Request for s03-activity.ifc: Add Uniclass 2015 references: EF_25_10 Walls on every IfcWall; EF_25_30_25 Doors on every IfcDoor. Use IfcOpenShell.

First a look at what the model holds.

```python
import ifcopenshell

model = ifcopenshell.open("s03-activity.ifc")
print(model.schema)
print("classifications:", [c.Name for c in model.by_type("IfcClassification")])
for ifc_class in ("IfcDoor", "IfcRoof", "IfcStair", "IfcWall", "IfcWindow"):
    print(ifc_class, len(model.by_type(ifc_class)))
```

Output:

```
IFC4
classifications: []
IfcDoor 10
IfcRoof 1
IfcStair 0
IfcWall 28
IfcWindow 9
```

```python
import ifcopenshell
import ifcopenshell.api.classification

model = ifcopenshell.open("s03-activity.ifc")

system = ifcopenshell.api.classification.add_classification(model, classification="Uniclass 2015")

codes = {
    "IfcWall": ("EF_25_10", "Walls"),
    "IfcDoor": ("EF_25_30_25", "Doors"),
}
for ifc_class, (code, name) in codes.items():
    products = model.by_type(ifc_class)
    ifcopenshell.api.classification.add_reference(
        model, products=products, classification=system, identification=code, name=name
    )
    print(code, len(products))

model.write("s03-activity_edited.ifc")
```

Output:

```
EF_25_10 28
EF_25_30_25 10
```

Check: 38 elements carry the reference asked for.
